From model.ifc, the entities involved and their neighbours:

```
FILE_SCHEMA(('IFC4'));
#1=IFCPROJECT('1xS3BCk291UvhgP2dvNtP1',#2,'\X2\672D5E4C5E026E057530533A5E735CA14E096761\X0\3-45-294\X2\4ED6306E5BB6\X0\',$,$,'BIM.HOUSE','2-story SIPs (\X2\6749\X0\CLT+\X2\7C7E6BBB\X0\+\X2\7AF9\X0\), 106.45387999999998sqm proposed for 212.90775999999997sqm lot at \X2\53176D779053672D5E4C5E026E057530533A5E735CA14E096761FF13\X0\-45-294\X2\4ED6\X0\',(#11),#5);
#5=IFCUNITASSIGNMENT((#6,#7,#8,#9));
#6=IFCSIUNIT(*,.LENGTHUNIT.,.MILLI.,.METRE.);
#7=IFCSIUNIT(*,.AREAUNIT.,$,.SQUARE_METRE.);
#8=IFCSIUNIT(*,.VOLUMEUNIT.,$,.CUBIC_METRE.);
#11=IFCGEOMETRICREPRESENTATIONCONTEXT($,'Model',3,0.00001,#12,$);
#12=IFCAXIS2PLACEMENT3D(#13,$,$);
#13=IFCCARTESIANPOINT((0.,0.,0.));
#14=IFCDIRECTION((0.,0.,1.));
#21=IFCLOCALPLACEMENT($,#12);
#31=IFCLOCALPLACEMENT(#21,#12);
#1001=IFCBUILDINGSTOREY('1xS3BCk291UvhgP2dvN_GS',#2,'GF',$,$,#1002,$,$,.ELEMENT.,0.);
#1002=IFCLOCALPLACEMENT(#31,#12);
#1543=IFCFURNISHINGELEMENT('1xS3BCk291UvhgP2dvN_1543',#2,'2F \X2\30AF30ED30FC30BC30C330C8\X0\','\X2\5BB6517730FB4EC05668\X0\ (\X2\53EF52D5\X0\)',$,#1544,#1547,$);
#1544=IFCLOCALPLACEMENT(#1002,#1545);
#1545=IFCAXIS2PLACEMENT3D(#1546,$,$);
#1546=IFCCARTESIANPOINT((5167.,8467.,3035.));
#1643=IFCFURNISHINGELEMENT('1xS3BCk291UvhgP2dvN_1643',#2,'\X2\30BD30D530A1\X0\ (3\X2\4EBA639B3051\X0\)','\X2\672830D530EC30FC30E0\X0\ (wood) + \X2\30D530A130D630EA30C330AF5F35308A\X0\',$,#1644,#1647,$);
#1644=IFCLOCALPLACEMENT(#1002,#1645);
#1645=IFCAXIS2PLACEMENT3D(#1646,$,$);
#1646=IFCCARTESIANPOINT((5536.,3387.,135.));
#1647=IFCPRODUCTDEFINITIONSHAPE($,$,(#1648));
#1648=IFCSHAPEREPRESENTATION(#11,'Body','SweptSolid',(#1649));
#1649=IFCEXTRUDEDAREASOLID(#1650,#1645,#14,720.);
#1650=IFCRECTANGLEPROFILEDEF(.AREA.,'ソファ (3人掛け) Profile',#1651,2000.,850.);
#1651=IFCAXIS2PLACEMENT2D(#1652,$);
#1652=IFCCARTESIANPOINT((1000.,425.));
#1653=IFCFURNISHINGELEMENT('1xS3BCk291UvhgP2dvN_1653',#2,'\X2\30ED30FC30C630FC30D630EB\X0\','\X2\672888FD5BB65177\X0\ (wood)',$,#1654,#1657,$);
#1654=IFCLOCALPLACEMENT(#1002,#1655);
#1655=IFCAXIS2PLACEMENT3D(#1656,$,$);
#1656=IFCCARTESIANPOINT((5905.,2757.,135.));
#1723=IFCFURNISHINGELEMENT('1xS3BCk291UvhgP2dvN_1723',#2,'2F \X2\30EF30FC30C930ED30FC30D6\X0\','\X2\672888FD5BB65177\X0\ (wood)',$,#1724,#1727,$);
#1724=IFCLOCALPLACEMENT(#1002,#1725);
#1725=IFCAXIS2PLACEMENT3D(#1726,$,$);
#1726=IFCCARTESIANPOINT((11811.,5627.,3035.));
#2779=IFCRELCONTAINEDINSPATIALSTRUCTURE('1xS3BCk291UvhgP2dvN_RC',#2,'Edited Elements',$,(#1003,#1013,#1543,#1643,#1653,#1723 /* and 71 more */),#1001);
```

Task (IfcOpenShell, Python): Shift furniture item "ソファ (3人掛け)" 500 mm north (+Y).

```python
import ifcopenshell
import ifcopenshell.api.geometry
import ifcopenshell.util.placement

model = ifcopenshell.open("model.ifc")

item = model.by_guid("1xS3BCk291UvhgP2dvN_1643")
matrix = ifcopenshell.util.placement.get_local_placement(item.ObjectPlacement)
matrix[1, 3] += 500.0
ifcopenshell.api.geometry.edit_object_placement(model, product=item, matrix=matrix, is_si=False)

print(ifcopenshell.util.placement.get_local_placement(item.ObjectPlacement).round(3) + 0.0)

model.write("model_rev.ifc")
```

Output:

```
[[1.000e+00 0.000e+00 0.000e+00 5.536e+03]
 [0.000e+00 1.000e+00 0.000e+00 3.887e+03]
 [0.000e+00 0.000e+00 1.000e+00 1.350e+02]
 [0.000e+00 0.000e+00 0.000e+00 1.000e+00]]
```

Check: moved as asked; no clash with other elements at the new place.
